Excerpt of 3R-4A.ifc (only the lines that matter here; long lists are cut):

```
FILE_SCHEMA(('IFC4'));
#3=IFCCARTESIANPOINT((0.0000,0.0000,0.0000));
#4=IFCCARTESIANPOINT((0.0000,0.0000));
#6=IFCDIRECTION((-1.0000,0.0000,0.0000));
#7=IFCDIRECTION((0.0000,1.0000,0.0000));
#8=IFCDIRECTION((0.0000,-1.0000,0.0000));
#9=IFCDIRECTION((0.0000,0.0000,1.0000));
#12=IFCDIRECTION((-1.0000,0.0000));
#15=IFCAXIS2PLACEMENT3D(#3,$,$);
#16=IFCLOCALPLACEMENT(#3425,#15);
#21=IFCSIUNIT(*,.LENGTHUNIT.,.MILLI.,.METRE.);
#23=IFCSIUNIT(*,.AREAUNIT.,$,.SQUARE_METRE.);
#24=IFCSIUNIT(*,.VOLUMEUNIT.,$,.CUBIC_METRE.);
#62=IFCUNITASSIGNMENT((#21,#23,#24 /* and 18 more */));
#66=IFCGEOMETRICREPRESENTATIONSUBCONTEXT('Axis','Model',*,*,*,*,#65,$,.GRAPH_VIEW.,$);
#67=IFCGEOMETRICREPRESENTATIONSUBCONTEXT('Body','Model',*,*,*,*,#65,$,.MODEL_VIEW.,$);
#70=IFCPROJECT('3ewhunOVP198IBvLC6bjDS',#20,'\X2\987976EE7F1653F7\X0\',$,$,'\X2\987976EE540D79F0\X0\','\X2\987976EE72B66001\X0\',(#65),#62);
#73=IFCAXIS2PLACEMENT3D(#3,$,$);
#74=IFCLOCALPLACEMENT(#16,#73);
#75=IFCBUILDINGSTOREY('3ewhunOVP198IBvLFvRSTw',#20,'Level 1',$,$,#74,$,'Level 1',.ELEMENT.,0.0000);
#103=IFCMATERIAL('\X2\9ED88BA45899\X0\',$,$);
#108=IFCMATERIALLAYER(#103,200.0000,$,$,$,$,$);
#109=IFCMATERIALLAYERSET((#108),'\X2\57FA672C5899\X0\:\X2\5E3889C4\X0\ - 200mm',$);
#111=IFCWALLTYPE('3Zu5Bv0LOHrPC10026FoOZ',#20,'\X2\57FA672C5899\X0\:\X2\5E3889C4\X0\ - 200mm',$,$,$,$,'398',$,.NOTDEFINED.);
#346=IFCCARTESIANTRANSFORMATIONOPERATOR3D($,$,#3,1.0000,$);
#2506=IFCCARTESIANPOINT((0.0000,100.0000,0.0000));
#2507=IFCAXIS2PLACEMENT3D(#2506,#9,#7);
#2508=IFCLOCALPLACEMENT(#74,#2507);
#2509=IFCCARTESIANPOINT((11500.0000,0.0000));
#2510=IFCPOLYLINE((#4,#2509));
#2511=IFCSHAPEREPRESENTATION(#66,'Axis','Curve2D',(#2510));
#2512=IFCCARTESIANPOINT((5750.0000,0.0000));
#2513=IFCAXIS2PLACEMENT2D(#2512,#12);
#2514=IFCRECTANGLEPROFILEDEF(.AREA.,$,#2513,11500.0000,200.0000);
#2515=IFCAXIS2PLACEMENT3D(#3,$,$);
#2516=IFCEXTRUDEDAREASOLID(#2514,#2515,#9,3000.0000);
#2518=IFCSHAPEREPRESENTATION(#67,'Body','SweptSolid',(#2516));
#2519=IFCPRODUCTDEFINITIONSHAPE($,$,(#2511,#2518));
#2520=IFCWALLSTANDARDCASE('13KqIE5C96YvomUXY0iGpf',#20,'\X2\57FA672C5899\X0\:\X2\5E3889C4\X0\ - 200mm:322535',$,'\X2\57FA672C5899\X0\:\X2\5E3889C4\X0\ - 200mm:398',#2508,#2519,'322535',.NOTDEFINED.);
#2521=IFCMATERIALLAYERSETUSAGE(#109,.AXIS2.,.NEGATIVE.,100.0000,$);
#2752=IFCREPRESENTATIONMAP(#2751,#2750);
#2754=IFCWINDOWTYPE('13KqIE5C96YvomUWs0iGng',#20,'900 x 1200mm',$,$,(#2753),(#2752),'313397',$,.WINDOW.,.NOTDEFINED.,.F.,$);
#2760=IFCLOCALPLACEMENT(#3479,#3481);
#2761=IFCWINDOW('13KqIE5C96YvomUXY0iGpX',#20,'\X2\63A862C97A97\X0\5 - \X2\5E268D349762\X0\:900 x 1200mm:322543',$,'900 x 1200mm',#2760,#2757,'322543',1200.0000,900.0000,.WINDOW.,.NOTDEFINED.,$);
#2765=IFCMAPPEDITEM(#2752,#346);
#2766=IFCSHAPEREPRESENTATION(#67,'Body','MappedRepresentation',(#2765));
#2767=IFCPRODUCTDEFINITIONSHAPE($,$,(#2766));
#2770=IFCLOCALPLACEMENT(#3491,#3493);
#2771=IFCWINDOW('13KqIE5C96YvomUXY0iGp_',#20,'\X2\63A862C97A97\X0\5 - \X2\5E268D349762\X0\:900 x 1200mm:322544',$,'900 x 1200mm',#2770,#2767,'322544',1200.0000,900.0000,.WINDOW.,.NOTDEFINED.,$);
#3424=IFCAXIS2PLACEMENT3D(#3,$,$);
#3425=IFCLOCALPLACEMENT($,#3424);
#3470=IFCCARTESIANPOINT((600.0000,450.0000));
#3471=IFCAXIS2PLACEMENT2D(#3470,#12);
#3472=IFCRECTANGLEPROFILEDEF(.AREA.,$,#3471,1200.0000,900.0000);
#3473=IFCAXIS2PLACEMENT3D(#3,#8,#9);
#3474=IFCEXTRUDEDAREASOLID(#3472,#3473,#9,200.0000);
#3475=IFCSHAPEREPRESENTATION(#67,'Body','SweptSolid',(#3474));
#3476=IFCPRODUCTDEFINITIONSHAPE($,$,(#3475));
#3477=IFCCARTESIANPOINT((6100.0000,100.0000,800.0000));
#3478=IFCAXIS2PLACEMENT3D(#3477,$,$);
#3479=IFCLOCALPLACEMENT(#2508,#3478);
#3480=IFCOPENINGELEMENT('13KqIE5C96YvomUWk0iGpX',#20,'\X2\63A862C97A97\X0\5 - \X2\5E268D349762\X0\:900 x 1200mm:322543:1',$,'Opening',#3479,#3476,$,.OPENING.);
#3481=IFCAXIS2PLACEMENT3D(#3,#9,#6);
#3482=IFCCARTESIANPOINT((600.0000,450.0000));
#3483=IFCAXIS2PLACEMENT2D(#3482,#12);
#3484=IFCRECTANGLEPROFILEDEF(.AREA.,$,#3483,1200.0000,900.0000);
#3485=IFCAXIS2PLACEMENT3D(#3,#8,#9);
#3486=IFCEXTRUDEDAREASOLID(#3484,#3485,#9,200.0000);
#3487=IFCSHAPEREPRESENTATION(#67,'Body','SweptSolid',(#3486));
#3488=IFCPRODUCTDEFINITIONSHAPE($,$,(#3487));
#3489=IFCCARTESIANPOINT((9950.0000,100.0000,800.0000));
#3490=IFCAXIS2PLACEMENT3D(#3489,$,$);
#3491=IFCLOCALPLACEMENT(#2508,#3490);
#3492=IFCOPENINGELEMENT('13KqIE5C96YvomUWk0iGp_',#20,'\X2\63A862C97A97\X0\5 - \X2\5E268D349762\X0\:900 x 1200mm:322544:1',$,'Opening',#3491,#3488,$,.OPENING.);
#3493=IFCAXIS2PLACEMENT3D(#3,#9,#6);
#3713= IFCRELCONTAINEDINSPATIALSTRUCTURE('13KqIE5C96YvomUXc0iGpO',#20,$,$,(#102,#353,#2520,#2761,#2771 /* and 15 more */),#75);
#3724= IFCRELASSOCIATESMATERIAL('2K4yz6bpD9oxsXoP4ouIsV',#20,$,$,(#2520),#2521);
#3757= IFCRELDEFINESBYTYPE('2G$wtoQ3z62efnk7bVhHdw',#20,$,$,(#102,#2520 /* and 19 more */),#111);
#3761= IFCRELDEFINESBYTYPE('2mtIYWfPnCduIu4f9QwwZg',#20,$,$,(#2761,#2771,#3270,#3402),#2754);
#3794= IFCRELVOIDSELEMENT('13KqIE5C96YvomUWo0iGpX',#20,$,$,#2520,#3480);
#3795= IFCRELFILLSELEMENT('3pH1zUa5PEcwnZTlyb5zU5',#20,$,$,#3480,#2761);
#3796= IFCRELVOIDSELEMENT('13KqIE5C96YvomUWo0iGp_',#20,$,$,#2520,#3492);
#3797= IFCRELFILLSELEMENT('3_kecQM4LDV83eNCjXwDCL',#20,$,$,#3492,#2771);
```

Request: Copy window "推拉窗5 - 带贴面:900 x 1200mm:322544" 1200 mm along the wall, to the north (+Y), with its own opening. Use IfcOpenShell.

```python
import ifcopenshell
import ifcopenshell.api.feature
import ifcopenshell.api.geometry
import ifcopenshell.api.root
import ifcopenshell.geom
import ifcopenshell.util.element
import ifcopenshell.util.placement
import ifcopenshell.util.shape
import ifcopenshell.util.unit

model = ifcopenshell.open("3R-4A.ifc")
unit_scale = ifcopenshell.util.unit.calculate_unit_scale(model)
settings = ifcopenshell.geom.settings()


def volume(element):
    """Net volume in cubic metres, openings subtracted."""
    shape = ifcopenshell.geom.create_shape(settings, element)
    return ifcopenshell.util.shape.get_volume(shape.geometry)


def reuse_history(source, copy):
    """copy_class also copies each property set's owner history, people and application; keep the originals."""
    for rel in copy.IsDefinedBy:
        if rel.is_a("IfcRelDefinesByProperties") and (history := rel.RelatingPropertyDefinition.OwnerHistory):
            rel.RelatingPropertyDefinition.OwnerHistory = source.OwnerHistory
            ifcopenshell.util.element.remove_deep2(model, history)


window = model.by_guid("13KqIE5C96YvomUXY0iGp_")
opening = window.FillsVoids[0].RelatingOpeningElement
wall = opening.VoidsElements[0].RelatingBuildingElement
before = volume(wall)
shift = ifcopenshell.util.placement.get_local_placement(wall.ObjectPlacement)[:3, 0] * 1.2 / unit_scale

# copy_class copies the void relationship, type, container and properties, but no geometry.
new_opening = ifcopenshell.api.root.copy_class(model, product=opening)
new_opening.Representation = ifcopenshell.util.element.copy_deep(
    model, opening.Representation, exclude=["IfcGeometricRepresentationContext", "IfcRepresentationMap"]
)
new_opening.Name = "推拉窗5 - 带贴面:900 x 1200mm"
new_window = ifcopenshell.api.root.copy_class(model, product=window)
new_window.Representation = ifcopenshell.util.element.copy_deep(
    model, window.Representation, exclude=["IfcGeometricRepresentationContext", "IfcRepresentationMap"]
)
new_window.Name = "推拉窗5 - 带贴面:900 x 1200mm"
new_window.Tag = None
reuse_history(window, new_window)
ifcopenshell.api.feature.add_filling(model, opening=new_opening, element=new_window)

for old, new in ((opening, new_opening), (window, new_window)):
    matrix = ifcopenshell.util.placement.get_local_placement(old.ObjectPlacement)
    matrix[:3, 3] += shift
    ifcopenshell.api.geometry.edit_object_placement(model, product=new, matrix=matrix, is_si=False)

after = volume(wall)

print(f"wall volume {before:.3f} -> {after:.3f} m3")

model.write("3R-4A_v2.ifc")
```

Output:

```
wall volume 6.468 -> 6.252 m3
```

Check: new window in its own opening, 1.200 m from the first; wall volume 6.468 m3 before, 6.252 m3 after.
